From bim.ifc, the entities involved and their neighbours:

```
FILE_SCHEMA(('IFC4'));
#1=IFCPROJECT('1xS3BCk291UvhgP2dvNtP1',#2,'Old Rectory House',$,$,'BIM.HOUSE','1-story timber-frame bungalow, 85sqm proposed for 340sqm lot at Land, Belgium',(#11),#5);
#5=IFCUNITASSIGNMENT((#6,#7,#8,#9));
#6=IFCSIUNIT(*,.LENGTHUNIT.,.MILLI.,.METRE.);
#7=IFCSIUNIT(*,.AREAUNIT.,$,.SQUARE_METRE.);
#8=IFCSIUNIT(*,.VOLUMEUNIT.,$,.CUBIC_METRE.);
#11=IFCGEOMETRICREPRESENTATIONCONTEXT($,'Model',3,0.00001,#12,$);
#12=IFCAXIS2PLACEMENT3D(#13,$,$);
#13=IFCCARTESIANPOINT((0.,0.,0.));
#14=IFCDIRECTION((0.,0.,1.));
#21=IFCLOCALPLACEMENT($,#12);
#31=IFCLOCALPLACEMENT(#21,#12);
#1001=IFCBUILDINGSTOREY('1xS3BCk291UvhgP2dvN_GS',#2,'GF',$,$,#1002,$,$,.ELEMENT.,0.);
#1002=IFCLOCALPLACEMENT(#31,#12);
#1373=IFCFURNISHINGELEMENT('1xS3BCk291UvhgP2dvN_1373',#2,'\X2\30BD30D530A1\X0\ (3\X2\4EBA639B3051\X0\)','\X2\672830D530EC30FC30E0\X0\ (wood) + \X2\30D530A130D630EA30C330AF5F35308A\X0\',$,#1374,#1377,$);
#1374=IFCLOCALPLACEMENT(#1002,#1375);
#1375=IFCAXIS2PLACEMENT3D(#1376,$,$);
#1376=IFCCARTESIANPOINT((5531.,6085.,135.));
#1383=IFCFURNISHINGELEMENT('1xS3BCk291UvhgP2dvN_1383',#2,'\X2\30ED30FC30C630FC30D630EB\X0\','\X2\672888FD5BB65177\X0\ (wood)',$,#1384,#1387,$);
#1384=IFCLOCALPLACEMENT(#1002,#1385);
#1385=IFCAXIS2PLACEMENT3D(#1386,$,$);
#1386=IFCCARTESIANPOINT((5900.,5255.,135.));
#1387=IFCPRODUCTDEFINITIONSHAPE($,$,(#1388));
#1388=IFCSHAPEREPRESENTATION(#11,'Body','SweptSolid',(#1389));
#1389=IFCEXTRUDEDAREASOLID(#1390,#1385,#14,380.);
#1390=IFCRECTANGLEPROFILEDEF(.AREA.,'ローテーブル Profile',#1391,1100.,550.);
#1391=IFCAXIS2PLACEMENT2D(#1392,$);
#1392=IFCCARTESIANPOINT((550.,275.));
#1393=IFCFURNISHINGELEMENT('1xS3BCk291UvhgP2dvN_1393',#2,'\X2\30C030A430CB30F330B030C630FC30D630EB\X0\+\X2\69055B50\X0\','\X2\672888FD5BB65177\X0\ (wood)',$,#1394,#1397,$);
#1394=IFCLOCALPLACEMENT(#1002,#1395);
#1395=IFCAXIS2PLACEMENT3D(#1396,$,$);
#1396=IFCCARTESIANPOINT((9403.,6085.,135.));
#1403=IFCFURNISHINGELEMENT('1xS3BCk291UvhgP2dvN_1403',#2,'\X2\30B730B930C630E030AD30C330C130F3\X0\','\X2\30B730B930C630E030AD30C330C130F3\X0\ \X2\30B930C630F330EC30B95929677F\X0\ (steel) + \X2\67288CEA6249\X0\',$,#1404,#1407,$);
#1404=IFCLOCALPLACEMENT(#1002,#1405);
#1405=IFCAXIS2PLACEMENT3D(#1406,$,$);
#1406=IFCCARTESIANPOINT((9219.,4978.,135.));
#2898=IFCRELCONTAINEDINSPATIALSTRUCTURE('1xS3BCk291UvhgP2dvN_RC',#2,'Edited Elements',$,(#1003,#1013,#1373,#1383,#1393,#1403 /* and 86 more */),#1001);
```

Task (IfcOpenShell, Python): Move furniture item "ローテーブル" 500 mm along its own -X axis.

```python
import ifcopenshell
import ifcopenshell.api.geometry
import ifcopenshell.util.placement

model = ifcopenshell.open("bim.ifc")

item = model.by_guid("1xS3BCk291UvhgP2dvN_1383")
matrix = ifcopenshell.util.placement.get_local_placement(item.ObjectPlacement)
matrix[:3, 3] -= matrix[:3, 0] * 500.0
ifcopenshell.api.geometry.edit_object_placement(model, product=item, matrix=matrix, is_si=False)

print(ifcopenshell.util.placement.get_local_placement(item.ObjectPlacement).round(3) + 0.0)

model.write("bim_updated.ifc")
```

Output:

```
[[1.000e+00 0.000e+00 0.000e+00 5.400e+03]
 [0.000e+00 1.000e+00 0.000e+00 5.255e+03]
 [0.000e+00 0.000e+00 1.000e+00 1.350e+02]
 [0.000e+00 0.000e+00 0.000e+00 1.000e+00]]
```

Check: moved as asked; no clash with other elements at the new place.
